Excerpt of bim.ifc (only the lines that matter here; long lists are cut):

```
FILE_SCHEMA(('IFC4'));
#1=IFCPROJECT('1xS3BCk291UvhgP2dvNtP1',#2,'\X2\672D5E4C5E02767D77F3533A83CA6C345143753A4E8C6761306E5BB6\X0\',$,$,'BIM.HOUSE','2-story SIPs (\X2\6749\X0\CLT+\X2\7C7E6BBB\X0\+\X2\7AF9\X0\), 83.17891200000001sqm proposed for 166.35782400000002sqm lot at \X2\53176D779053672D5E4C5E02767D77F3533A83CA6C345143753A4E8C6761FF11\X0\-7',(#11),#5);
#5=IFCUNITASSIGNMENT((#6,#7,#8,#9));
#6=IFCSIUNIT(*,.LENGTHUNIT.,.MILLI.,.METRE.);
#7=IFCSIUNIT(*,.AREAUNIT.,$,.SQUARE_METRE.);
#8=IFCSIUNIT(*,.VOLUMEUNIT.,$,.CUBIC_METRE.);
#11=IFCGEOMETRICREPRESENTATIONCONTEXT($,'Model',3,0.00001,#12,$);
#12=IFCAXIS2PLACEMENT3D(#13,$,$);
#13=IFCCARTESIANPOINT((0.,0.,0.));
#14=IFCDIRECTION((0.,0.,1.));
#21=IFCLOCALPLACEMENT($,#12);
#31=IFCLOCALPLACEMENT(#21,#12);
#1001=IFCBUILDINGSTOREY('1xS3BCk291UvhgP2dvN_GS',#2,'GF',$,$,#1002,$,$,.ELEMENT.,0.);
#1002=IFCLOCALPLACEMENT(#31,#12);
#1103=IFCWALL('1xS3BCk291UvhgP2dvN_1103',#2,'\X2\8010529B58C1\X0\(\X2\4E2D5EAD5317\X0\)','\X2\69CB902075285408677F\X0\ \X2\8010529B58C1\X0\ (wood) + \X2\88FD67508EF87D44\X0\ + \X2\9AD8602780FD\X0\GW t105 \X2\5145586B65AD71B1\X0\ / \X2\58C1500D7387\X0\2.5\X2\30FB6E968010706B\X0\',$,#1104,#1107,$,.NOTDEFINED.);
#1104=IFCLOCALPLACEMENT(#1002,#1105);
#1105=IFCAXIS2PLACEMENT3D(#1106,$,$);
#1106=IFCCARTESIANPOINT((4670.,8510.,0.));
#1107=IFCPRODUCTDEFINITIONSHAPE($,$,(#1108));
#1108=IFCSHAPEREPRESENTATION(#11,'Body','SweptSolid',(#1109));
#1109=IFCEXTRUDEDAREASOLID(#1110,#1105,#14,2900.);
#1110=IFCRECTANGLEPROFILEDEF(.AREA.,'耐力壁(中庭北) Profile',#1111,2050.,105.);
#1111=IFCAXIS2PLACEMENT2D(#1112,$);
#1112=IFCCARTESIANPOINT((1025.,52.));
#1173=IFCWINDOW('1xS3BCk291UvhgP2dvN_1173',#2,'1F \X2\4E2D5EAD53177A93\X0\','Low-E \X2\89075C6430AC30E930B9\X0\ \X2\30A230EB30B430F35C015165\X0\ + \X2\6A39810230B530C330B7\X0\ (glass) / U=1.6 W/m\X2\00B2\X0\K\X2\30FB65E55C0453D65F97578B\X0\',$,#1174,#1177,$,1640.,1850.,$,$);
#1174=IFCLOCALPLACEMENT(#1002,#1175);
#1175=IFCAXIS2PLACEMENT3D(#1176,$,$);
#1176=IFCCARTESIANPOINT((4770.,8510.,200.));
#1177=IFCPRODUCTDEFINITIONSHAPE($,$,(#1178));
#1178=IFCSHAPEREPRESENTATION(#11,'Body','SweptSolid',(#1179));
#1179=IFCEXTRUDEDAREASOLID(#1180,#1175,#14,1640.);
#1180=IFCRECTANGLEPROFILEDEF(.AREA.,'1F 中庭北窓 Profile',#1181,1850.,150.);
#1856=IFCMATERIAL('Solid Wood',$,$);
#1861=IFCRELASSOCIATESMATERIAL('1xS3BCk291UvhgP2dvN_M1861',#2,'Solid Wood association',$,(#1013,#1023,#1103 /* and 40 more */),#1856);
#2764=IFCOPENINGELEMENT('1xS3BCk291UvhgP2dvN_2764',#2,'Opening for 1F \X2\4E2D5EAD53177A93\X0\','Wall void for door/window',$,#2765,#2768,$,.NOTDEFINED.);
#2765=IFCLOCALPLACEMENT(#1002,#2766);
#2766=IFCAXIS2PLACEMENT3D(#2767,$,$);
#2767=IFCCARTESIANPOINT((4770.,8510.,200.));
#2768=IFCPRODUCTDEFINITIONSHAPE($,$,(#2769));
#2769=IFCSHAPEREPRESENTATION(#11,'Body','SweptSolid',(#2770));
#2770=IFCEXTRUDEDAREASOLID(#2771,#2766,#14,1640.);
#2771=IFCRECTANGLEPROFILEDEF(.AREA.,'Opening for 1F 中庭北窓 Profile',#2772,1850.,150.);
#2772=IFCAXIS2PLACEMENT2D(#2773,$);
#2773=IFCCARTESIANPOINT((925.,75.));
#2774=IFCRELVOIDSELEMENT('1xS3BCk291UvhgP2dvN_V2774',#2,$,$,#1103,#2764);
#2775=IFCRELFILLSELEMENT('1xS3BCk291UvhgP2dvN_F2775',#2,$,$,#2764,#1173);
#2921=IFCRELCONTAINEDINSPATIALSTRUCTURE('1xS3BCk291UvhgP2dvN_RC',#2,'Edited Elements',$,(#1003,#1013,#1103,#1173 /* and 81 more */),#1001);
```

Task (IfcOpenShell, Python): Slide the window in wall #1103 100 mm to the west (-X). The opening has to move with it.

```python
import ifcopenshell
import ifcopenshell.api.geometry
import ifcopenshell.util.placement

model = ifcopenshell.open("bim.ifc")

window = model.by_guid("1xS3BCk291UvhgP2dvN_1173")
opening = window.FillsVoids[0].RelatingOpeningElement
wall = opening.VoidsElements[0].RelatingBuildingElement

wall_matrix = ifcopenshell.util.placement.get_local_placement(wall.ObjectPlacement)
shift = wall_matrix[:3, 0] * -100.0
before = ifcopenshell.util.placement.get_local_placement(window.ObjectPlacement)[:3, 3].copy()

# The window is not placed relative to its opening, so move both.
for product in (opening, window):
    matrix = ifcopenshell.util.placement.get_local_placement(product.ObjectPlacement)
    matrix[:3, 3] += shift
    ifcopenshell.api.geometry.edit_object_placement(model, product=product, matrix=matrix, is_si=False)

after = ifcopenshell.util.placement.get_local_placement(window.ObjectPlacement)[:3, 3]
print("window moved by", (after - before).round(3) + 0.0)

model.write("bim_v2.ifc")
```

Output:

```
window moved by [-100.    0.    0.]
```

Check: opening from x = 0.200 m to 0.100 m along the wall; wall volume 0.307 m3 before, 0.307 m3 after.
